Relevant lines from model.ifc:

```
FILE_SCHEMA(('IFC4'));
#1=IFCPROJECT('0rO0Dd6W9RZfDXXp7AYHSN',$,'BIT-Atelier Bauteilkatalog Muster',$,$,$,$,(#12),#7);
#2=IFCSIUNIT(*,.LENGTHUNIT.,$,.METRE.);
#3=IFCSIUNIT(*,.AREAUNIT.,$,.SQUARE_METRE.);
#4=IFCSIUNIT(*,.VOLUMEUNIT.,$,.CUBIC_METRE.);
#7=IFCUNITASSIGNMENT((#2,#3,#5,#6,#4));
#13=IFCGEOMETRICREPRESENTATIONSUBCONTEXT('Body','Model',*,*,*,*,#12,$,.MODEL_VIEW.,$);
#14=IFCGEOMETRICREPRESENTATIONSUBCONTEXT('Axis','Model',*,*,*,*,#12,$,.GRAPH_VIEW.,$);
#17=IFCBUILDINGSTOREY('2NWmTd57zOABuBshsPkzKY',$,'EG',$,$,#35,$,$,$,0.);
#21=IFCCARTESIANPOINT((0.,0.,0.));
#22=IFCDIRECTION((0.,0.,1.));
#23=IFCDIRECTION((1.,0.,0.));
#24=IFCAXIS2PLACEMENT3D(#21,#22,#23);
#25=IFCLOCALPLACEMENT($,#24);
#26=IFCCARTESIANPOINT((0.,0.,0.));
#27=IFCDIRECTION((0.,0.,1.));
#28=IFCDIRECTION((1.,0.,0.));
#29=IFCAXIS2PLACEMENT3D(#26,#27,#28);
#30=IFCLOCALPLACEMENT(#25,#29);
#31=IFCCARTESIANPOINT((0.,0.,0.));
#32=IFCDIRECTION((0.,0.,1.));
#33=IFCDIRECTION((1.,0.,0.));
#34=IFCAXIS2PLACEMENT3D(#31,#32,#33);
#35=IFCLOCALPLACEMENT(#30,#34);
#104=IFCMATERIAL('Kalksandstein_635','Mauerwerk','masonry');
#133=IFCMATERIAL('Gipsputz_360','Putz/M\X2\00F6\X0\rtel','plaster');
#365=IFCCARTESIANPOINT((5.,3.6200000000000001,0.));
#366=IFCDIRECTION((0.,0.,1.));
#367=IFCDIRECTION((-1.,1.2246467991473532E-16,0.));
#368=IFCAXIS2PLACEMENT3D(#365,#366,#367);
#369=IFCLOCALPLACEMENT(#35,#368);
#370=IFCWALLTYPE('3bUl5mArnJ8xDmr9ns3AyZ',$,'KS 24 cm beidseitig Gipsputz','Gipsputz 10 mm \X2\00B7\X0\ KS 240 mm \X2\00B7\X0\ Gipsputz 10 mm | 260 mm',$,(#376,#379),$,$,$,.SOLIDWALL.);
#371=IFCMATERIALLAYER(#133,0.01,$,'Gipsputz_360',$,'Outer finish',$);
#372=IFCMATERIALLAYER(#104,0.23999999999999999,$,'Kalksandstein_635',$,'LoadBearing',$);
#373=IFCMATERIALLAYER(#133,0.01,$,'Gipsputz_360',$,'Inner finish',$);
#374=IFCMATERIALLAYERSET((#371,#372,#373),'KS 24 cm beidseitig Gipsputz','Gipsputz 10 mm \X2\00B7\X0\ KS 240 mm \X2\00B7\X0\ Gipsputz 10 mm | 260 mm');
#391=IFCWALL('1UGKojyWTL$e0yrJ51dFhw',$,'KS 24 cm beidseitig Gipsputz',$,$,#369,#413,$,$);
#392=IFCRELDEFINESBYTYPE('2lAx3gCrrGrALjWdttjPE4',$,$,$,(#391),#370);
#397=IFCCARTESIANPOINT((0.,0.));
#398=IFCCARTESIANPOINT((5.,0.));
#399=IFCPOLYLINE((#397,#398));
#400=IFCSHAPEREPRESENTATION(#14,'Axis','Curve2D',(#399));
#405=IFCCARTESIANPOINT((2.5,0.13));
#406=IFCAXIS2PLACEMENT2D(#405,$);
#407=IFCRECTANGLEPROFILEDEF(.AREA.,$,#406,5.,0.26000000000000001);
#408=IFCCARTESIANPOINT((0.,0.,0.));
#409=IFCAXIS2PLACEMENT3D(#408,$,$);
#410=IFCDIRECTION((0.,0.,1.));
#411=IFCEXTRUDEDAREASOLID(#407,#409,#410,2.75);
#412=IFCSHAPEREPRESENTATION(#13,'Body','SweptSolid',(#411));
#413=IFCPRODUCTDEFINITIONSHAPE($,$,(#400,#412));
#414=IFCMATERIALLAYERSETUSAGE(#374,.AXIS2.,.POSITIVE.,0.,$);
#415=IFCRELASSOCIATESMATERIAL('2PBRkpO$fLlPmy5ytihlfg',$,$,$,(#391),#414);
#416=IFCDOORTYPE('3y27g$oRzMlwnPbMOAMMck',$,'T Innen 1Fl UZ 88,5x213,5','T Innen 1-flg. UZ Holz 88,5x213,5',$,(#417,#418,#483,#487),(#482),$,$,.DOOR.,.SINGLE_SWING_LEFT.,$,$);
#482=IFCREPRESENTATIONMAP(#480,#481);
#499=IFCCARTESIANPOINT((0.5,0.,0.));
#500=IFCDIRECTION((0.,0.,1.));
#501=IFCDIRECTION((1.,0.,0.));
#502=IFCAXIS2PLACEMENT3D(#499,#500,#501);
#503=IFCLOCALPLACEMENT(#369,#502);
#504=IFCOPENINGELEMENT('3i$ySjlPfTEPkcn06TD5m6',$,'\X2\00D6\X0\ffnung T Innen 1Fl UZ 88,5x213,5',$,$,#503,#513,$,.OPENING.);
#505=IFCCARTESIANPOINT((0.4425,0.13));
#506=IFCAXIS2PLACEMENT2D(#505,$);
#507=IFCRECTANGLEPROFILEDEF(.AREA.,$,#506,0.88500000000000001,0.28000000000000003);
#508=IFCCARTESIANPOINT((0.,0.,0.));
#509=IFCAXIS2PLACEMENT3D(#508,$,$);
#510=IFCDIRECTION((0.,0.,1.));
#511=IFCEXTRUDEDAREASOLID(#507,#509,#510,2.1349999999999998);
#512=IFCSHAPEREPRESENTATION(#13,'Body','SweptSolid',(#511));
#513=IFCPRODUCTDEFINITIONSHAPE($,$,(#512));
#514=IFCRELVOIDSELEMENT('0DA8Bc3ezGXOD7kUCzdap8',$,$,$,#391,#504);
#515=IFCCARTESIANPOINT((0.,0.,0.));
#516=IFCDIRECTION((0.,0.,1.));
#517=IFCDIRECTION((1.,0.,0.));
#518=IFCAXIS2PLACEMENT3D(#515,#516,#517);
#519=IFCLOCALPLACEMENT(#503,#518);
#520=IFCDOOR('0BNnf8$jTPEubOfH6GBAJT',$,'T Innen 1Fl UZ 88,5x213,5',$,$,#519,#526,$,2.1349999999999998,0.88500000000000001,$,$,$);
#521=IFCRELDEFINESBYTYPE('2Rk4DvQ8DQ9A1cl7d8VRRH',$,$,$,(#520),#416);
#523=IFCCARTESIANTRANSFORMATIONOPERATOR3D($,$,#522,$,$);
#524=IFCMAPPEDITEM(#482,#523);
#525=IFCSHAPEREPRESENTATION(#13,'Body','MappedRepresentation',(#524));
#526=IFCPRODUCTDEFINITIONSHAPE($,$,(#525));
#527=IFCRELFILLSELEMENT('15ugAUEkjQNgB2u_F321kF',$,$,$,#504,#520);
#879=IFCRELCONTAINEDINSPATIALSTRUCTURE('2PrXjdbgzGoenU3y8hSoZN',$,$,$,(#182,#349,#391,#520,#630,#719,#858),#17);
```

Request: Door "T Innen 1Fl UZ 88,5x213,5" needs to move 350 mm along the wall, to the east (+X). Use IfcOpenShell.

```python
import ifcopenshell
import ifcopenshell.api.geometry
import ifcopenshell.util.placement
import ifcopenshell.util.unit

model = ifcopenshell.open("model.ifc")
unit_scale = ifcopenshell.util.unit.calculate_unit_scale(model)

door = model.by_guid("0BNnf8$jTPEubOfH6GBAJT")
opening = door.FillsVoids[0].RelatingOpeningElement
wall = opening.VoidsElements[0].RelatingBuildingElement

wall_matrix = ifcopenshell.util.placement.get_local_placement(wall.ObjectPlacement)
shift = wall_matrix[:3, 0] * -0.35 / unit_scale
before = ifcopenshell.util.placement.get_local_placement(door.ObjectPlacement)[:3, 3].copy()

# The door is placed relative to its opening, so it follows when the opening moves.
matrix = ifcopenshell.util.placement.get_local_placement(opening.ObjectPlacement)
matrix[:3, 3] += shift
ifcopenshell.api.geometry.edit_object_placement(
    model, product=opening, matrix=matrix, is_si=False, should_transform_children=True
)

after = ifcopenshell.util.placement.get_local_placement(door.ObjectPlacement)[:3, 3]
print("door moved by", (after - before).round(3) + 0.0)

model.write("model_rev.ifc")
```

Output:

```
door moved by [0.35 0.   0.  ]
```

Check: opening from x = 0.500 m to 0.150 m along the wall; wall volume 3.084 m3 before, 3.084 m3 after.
